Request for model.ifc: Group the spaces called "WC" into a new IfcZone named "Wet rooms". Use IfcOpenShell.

First a look at what the model holds.

```python
import ifcopenshell

model = ifcopenshell.open("model.ifc")
print(model.schema)
seen = {}
for space in model.by_type("IfcSpace"):
    seen[space.LongName] = seen.get(space.LongName, 0) + 1
for name, count in sorted(seen.items(), key=str):
    print(count, "x", name)
print("zones:", [z.Name for z in model.by_type("IfcZone")][:20])
```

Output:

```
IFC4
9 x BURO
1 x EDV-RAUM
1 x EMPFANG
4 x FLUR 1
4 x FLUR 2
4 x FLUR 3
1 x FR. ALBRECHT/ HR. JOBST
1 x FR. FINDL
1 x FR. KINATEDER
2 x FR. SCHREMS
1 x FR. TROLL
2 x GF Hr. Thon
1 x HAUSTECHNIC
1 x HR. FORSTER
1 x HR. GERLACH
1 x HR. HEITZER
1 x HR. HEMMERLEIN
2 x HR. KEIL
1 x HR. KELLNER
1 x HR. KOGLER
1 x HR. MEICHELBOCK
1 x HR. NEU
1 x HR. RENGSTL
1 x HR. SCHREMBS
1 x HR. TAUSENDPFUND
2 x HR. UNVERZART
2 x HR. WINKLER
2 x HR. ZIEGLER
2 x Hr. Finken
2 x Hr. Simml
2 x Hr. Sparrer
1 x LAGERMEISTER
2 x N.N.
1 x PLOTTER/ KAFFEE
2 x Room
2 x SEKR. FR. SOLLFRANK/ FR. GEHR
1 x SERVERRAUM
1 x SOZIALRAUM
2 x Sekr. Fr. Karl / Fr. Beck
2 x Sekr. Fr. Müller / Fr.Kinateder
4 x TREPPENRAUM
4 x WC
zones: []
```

```python
import ifcopenshell
import ifcopenshell.api.group
import ifcopenshell.api.root

model = ifcopenshell.open("model.ifc")

names = {"WC"}
spaces = [s for s in model.by_type("IfcSpace") if s.LongName in names]

zone = ifcopenshell.api.root.create_entity(model, ifc_class="IfcZone", name="Wet rooms")
ifcopenshell.api.group.assign_group(model, products=spaces, group=zone)
print(len(spaces), "spaces in", zone.Name)

model.write("model_updated.ifc")
```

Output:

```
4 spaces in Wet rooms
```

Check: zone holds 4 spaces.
